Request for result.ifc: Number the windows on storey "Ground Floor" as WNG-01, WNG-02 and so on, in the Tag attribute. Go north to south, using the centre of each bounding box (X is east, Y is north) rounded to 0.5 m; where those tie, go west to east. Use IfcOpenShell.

First a look at what the model holds.

```python
import ifcopenshell
import ifcopenshell.util.element
import ifcopenshell.util.placement

model = ifcopenshell.open("result.ifc")
print(model.schema)
storey = next(s for s in model.by_type("IfcBuildingStorey") if s.Name == "Ground Floor")
windows = [e for e in ifcopenshell.util.element.get_decomposition(storey) if e.is_a("IfcWindow")]
for e in sorted(windows, key=lambda e: e.id()):
    origin = ifcopenshell.util.placement.get_local_placement(e.ObjectPlacement)[:3, 3]
    print(e.id(), e.Tag, e.Name, origin.round(2) + 0.0, sep=" | ")
```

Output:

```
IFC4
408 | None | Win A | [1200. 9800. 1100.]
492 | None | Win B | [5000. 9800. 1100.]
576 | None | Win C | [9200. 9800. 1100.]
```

```python
import ifcopenshell
import ifcopenshell.geom
import ifcopenshell.util.element
import ifcopenshell.util.shape

model = ifcopenshell.open("result.ifc")
settings = ifcopenshell.geom.settings()
settings.set("use-world-coords", True)


def centre(element):
    shape = ifcopenshell.geom.create_shape(settings, element)
    return ifcopenshell.util.shape.get_bbox_centroid(shape.geometry)


storey = next(s for s in model.by_type("IfcBuildingStorey") if s.Name == "Ground Floor")
windows = [e for e in ifcopenshell.util.element.get_decomposition(storey) if e.is_a("IfcWindow")]

# Insertion points can sit at a corner or the storey origin, so sort by the geometry (in metres).
centres = {e: centre(e) for e in windows}
windows.sort(key=lambda e: (-round(centres[e][1] / 0.5), centres[e][0]))

for i, e in enumerate(windows, start=1):
    number = f"WNG-{i:02d}"
    e.Tag = number
    print(e.id(), number)

model.write("result_v2.ifc")
```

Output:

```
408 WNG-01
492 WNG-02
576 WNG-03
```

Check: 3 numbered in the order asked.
